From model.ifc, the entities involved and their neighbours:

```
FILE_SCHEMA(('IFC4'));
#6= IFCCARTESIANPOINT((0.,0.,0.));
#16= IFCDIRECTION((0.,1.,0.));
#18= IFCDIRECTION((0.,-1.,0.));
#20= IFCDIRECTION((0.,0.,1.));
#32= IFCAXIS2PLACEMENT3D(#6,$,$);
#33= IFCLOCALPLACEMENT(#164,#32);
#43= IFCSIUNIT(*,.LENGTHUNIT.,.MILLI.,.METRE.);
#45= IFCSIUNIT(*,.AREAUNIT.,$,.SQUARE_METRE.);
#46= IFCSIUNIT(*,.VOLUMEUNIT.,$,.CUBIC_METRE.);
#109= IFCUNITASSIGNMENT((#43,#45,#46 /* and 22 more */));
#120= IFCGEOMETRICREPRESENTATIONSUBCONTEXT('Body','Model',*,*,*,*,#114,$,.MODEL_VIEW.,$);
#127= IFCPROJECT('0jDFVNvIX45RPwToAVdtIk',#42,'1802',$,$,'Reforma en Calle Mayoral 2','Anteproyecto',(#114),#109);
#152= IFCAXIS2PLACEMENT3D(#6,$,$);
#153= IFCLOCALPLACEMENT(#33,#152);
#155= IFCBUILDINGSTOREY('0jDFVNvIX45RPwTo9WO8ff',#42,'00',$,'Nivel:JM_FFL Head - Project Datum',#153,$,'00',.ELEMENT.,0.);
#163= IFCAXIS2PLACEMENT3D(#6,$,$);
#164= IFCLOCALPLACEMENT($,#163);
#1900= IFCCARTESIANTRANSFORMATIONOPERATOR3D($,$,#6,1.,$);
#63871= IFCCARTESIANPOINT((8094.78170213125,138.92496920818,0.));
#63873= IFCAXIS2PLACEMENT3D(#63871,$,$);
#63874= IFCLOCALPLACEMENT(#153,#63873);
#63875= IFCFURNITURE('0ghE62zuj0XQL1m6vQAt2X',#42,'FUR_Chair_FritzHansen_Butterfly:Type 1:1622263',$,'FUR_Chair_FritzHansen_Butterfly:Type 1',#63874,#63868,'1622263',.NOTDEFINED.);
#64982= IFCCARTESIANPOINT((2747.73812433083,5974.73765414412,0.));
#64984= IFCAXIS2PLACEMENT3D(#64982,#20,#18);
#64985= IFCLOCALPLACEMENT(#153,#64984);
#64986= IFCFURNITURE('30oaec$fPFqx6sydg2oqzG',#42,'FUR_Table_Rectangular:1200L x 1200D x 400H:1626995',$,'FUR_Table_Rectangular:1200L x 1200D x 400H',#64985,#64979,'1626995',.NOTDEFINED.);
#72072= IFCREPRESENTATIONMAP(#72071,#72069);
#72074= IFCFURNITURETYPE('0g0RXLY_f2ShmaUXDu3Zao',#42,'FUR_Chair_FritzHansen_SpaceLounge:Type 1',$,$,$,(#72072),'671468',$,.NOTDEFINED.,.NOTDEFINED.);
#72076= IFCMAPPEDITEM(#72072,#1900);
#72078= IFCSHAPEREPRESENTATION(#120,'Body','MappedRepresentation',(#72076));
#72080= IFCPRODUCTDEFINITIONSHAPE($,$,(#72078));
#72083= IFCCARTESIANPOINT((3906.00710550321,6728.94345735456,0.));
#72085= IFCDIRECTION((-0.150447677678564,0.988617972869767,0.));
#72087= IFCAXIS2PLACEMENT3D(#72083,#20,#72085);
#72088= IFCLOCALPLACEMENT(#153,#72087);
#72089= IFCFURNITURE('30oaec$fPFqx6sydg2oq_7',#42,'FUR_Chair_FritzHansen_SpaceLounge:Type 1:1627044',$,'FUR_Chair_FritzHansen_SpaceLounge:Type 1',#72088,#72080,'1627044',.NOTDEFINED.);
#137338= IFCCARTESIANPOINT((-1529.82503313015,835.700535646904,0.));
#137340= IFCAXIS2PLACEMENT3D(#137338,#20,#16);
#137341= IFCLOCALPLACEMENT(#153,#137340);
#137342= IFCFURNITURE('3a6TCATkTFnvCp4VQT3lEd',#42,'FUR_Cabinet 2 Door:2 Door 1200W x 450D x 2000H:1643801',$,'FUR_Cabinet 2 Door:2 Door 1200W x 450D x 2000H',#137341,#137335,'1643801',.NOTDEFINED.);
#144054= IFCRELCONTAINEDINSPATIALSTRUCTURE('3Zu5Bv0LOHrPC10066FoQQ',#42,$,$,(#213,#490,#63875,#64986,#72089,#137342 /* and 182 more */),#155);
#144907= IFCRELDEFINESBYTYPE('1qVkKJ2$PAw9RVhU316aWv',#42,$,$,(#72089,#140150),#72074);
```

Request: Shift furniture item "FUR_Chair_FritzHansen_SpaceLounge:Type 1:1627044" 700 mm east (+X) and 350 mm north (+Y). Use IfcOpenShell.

```python
import ifcopenshell
import ifcopenshell.api.geometry
import ifcopenshell.util.placement

model = ifcopenshell.open("model.ifc")

item = model.by_guid("30oaec$fPFqx6sydg2oq_7")
matrix = ifcopenshell.util.placement.get_local_placement(item.ObjectPlacement)
matrix[0, 3] += 700.0
matrix[1, 3] += 350.0
ifcopenshell.api.geometry.edit_object_placement(model, product=item, matrix=matrix, is_si=False)

print(ifcopenshell.util.placement.get_local_placement(item.ObjectPlacement).round(3) + 0.0)

model.write("model_rev.ifc")
```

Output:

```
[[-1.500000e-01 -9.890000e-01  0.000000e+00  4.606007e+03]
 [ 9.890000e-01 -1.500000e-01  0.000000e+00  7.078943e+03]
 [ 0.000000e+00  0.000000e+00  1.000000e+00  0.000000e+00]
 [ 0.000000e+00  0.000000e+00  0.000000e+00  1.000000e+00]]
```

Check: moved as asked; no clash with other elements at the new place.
